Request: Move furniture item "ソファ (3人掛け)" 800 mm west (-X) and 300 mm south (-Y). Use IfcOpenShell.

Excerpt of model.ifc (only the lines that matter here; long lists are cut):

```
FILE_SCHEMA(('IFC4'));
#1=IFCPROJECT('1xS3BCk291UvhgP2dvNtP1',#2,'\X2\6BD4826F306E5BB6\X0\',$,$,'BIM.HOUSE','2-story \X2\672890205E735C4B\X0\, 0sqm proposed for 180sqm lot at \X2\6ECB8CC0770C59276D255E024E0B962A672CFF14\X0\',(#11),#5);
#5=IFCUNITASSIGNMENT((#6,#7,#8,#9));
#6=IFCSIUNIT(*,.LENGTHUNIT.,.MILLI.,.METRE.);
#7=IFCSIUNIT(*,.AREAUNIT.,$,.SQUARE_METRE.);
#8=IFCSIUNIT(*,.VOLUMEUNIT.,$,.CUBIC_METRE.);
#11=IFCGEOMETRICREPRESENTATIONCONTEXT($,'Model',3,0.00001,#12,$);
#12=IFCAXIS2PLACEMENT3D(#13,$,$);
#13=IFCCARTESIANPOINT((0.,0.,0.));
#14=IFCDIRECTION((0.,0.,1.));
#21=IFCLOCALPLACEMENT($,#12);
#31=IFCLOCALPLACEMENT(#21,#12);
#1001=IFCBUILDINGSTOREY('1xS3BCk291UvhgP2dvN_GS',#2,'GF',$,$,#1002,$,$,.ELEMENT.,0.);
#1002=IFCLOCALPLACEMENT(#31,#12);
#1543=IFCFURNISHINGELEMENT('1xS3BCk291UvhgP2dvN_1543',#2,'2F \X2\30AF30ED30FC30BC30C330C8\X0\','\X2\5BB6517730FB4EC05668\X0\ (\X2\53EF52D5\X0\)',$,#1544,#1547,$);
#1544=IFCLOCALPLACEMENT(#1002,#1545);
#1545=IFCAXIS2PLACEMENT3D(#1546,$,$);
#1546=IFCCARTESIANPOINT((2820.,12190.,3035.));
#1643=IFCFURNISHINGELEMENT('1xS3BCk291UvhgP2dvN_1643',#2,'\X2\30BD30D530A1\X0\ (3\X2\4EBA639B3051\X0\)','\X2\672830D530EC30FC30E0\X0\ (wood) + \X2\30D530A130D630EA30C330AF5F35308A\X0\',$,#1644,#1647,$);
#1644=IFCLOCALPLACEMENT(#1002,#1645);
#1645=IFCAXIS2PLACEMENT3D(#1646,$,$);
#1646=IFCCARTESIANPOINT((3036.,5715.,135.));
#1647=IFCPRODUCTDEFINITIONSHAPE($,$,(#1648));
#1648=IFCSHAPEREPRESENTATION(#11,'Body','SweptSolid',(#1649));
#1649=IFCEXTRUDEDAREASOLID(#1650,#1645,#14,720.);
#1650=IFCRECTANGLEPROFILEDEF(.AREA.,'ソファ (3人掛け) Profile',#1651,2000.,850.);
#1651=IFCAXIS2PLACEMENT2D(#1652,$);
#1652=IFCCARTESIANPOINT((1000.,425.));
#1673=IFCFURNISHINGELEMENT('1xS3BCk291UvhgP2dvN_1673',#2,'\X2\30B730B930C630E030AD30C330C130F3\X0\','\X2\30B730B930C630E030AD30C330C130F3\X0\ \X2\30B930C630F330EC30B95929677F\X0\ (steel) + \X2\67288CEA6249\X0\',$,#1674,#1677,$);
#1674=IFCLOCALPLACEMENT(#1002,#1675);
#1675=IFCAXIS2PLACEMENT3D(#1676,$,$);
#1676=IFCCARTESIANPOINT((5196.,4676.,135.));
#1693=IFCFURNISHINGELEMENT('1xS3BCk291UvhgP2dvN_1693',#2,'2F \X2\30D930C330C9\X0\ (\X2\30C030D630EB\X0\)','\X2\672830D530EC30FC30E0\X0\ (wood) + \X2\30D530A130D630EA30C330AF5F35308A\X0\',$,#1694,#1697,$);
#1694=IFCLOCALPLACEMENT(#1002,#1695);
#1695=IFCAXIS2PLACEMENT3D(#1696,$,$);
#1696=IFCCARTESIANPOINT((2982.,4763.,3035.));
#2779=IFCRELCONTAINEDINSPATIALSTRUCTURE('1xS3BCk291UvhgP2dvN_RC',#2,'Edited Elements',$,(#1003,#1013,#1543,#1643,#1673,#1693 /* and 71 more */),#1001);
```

```python
import ifcopenshell
import ifcopenshell.api.geometry
import ifcopenshell.util.placement

model = ifcopenshell.open("model.ifc")

item = model.by_id(1643)
matrix = ifcopenshell.util.placement.get_local_placement(item.ObjectPlacement)
matrix[0, 3] -= 800.0
matrix[1, 3] -= 300.0
ifcopenshell.api.geometry.edit_object_placement(model, product=item, matrix=matrix, is_si=False)

print(ifcopenshell.util.placement.get_local_placement(item.ObjectPlacement).round(3) + 0.0)

model.write("model_edited.ifc")
```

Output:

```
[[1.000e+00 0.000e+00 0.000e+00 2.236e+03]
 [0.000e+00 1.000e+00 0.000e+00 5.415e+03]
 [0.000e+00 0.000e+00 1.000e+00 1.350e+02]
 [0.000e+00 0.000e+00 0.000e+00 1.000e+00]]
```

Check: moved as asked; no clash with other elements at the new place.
